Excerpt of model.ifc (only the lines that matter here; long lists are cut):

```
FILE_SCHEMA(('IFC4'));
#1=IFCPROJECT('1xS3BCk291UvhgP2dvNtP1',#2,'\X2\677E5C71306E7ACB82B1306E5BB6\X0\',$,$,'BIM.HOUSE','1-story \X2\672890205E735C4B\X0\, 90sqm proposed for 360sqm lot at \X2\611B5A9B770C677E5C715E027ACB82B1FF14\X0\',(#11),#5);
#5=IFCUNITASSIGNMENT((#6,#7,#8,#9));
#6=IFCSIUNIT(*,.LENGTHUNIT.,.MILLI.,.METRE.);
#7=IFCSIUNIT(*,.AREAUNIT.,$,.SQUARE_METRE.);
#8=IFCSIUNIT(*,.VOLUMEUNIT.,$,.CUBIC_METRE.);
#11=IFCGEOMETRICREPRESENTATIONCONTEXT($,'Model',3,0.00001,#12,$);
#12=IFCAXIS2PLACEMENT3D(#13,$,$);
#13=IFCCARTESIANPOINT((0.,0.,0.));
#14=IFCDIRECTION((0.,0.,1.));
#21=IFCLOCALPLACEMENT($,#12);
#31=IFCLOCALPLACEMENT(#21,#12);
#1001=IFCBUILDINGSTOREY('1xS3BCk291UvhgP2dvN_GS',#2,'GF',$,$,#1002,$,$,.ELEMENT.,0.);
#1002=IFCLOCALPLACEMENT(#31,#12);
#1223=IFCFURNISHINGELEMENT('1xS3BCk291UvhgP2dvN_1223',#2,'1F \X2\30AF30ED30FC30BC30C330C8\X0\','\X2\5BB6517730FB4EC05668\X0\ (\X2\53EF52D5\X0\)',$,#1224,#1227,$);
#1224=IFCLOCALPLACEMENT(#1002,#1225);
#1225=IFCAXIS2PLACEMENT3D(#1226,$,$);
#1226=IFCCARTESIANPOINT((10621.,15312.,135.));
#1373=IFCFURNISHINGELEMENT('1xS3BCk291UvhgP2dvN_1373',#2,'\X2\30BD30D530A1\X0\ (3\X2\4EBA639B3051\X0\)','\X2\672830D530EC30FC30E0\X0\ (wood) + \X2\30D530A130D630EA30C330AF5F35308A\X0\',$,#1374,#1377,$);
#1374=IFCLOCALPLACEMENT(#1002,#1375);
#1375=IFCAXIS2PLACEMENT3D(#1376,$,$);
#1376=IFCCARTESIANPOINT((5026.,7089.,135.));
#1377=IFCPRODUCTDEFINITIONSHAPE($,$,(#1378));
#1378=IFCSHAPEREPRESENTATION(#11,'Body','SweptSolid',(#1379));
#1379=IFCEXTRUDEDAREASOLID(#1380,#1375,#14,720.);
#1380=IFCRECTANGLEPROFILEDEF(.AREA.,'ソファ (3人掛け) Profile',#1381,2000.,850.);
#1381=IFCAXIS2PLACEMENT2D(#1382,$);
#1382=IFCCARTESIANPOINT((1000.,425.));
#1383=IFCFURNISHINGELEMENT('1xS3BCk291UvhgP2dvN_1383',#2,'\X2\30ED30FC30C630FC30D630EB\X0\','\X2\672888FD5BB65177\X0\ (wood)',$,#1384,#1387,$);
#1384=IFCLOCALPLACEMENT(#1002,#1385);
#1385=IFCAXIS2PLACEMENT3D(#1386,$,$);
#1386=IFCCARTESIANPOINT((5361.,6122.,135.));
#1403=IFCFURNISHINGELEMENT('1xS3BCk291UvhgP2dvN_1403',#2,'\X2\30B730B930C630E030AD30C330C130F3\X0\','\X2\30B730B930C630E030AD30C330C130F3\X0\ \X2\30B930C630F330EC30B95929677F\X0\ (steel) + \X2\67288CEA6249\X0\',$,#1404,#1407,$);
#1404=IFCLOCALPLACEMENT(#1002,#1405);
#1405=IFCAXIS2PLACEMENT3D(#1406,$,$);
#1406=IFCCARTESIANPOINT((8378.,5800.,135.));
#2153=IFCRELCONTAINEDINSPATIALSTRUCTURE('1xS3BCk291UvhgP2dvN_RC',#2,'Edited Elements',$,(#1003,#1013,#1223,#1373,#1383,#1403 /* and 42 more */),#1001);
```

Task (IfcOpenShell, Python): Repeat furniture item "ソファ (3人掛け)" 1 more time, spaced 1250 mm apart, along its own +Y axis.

```python
import ifcopenshell
import ifcopenshell.api.geometry
import ifcopenshell.api.root
import ifcopenshell.util.element
import ifcopenshell.util.placement
import ifcopenshell.util.unit

model = ifcopenshell.open("model.ifc")
unit_scale = ifcopenshell.util.unit.calculate_unit_scale(model)


def reuse_history(source, copy):
    """copy_class also copies each property set's owner history, people and application; keep the originals."""
    for rel in copy.IsDefinedBy:
        if rel.is_a("IfcRelDefinesByProperties") and (history := rel.RelatingPropertyDefinition.OwnerHistory):
            rel.RelatingPropertyDefinition.OwnerHistory = source.OwnerHistory
            ifcopenshell.util.element.remove_deep2(model, history)


source = model.by_guid("1xS3BCk291UvhgP2dvN_1373")
base = ifcopenshell.util.placement.get_local_placement(source.ObjectPlacement)
step = base[:3, 1] * 1.25 / unit_scale

for i in range(1, 2):
    copy = ifcopenshell.api.root.copy_class(model, product=source)
    copy.Representation = ifcopenshell.util.element.copy_deep(
        model, source.Representation, exclude=["IfcGeometricRepresentationContext", "IfcRepresentationMap"]
    )
    reuse_history(source, copy)
    matrix = base.copy()
    matrix[:3, 3] += i * step
    print("added at", matrix[:3, 3].round(3) + 0.0)
    ifcopenshell.api.geometry.edit_object_placement(model, product=copy, matrix=matrix, is_si=False)

model.write("model_edited.ifc")
```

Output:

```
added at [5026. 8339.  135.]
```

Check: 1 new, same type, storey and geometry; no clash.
